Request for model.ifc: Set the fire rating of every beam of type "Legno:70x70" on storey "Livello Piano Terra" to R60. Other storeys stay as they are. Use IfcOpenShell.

First a look at what the model holds.

```python
import ifcopenshell
import ifcopenshell.util.element

model = ifcopenshell.open("model.ifc")
print(model.schema)
storey = next(s for s in model.by_type("IfcBuildingStorey") if s.Name == "Livello Piano Terra")
beams = [e for e in ifcopenshell.util.element.get_decomposition(storey) if e.is_a("IfcBeam")]
seen = {}
for e in beams:
    element_type = ifcopenshell.util.element.get_type(e)
    key = (element_type.Name if element_type != e and element_type else None, ifcopenshell.util.element.get_pset(e, "Pset_BeamCommon", "FireRating"))
    seen[key] = seen.get(key, 0) + 1
for (name, value), count in sorted(seen.items(), key=str):
    print(count, "x", name, "|", value)
```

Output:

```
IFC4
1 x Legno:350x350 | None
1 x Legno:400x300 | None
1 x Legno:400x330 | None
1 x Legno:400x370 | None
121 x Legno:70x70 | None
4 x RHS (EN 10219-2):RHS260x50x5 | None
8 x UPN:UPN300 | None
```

```python
import ifcopenshell
import ifcopenshell.api.pset
import ifcopenshell.util.element

model = ifcopenshell.open("model.ifc")

storey = next(s for s in model.by_type("IfcBuildingStorey") if s.Name == "Livello Piano Terra")
beams = [e for e in ifcopenshell.util.element.get_decomposition(storey) if e.is_a("IfcBeam")]

count = 0
for e in beams:
    element_type = ifcopenshell.util.element.get_type(e)
    if element_type in (None, e) or element_type.Name != "Legno:70x70":
        continue
    # add_pset returns the element's existing set when there is one.
    pset = ifcopenshell.api.pset.add_pset(model, product=e, name="Pset_BeamCommon")
    ifcopenshell.api.pset.edit_pset(model, pset=pset, properties={"FireRating": "R60"})
    count += 1

print(count, "beams updated")

model.write("model_edited.ifc")
```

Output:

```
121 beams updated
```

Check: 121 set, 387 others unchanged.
